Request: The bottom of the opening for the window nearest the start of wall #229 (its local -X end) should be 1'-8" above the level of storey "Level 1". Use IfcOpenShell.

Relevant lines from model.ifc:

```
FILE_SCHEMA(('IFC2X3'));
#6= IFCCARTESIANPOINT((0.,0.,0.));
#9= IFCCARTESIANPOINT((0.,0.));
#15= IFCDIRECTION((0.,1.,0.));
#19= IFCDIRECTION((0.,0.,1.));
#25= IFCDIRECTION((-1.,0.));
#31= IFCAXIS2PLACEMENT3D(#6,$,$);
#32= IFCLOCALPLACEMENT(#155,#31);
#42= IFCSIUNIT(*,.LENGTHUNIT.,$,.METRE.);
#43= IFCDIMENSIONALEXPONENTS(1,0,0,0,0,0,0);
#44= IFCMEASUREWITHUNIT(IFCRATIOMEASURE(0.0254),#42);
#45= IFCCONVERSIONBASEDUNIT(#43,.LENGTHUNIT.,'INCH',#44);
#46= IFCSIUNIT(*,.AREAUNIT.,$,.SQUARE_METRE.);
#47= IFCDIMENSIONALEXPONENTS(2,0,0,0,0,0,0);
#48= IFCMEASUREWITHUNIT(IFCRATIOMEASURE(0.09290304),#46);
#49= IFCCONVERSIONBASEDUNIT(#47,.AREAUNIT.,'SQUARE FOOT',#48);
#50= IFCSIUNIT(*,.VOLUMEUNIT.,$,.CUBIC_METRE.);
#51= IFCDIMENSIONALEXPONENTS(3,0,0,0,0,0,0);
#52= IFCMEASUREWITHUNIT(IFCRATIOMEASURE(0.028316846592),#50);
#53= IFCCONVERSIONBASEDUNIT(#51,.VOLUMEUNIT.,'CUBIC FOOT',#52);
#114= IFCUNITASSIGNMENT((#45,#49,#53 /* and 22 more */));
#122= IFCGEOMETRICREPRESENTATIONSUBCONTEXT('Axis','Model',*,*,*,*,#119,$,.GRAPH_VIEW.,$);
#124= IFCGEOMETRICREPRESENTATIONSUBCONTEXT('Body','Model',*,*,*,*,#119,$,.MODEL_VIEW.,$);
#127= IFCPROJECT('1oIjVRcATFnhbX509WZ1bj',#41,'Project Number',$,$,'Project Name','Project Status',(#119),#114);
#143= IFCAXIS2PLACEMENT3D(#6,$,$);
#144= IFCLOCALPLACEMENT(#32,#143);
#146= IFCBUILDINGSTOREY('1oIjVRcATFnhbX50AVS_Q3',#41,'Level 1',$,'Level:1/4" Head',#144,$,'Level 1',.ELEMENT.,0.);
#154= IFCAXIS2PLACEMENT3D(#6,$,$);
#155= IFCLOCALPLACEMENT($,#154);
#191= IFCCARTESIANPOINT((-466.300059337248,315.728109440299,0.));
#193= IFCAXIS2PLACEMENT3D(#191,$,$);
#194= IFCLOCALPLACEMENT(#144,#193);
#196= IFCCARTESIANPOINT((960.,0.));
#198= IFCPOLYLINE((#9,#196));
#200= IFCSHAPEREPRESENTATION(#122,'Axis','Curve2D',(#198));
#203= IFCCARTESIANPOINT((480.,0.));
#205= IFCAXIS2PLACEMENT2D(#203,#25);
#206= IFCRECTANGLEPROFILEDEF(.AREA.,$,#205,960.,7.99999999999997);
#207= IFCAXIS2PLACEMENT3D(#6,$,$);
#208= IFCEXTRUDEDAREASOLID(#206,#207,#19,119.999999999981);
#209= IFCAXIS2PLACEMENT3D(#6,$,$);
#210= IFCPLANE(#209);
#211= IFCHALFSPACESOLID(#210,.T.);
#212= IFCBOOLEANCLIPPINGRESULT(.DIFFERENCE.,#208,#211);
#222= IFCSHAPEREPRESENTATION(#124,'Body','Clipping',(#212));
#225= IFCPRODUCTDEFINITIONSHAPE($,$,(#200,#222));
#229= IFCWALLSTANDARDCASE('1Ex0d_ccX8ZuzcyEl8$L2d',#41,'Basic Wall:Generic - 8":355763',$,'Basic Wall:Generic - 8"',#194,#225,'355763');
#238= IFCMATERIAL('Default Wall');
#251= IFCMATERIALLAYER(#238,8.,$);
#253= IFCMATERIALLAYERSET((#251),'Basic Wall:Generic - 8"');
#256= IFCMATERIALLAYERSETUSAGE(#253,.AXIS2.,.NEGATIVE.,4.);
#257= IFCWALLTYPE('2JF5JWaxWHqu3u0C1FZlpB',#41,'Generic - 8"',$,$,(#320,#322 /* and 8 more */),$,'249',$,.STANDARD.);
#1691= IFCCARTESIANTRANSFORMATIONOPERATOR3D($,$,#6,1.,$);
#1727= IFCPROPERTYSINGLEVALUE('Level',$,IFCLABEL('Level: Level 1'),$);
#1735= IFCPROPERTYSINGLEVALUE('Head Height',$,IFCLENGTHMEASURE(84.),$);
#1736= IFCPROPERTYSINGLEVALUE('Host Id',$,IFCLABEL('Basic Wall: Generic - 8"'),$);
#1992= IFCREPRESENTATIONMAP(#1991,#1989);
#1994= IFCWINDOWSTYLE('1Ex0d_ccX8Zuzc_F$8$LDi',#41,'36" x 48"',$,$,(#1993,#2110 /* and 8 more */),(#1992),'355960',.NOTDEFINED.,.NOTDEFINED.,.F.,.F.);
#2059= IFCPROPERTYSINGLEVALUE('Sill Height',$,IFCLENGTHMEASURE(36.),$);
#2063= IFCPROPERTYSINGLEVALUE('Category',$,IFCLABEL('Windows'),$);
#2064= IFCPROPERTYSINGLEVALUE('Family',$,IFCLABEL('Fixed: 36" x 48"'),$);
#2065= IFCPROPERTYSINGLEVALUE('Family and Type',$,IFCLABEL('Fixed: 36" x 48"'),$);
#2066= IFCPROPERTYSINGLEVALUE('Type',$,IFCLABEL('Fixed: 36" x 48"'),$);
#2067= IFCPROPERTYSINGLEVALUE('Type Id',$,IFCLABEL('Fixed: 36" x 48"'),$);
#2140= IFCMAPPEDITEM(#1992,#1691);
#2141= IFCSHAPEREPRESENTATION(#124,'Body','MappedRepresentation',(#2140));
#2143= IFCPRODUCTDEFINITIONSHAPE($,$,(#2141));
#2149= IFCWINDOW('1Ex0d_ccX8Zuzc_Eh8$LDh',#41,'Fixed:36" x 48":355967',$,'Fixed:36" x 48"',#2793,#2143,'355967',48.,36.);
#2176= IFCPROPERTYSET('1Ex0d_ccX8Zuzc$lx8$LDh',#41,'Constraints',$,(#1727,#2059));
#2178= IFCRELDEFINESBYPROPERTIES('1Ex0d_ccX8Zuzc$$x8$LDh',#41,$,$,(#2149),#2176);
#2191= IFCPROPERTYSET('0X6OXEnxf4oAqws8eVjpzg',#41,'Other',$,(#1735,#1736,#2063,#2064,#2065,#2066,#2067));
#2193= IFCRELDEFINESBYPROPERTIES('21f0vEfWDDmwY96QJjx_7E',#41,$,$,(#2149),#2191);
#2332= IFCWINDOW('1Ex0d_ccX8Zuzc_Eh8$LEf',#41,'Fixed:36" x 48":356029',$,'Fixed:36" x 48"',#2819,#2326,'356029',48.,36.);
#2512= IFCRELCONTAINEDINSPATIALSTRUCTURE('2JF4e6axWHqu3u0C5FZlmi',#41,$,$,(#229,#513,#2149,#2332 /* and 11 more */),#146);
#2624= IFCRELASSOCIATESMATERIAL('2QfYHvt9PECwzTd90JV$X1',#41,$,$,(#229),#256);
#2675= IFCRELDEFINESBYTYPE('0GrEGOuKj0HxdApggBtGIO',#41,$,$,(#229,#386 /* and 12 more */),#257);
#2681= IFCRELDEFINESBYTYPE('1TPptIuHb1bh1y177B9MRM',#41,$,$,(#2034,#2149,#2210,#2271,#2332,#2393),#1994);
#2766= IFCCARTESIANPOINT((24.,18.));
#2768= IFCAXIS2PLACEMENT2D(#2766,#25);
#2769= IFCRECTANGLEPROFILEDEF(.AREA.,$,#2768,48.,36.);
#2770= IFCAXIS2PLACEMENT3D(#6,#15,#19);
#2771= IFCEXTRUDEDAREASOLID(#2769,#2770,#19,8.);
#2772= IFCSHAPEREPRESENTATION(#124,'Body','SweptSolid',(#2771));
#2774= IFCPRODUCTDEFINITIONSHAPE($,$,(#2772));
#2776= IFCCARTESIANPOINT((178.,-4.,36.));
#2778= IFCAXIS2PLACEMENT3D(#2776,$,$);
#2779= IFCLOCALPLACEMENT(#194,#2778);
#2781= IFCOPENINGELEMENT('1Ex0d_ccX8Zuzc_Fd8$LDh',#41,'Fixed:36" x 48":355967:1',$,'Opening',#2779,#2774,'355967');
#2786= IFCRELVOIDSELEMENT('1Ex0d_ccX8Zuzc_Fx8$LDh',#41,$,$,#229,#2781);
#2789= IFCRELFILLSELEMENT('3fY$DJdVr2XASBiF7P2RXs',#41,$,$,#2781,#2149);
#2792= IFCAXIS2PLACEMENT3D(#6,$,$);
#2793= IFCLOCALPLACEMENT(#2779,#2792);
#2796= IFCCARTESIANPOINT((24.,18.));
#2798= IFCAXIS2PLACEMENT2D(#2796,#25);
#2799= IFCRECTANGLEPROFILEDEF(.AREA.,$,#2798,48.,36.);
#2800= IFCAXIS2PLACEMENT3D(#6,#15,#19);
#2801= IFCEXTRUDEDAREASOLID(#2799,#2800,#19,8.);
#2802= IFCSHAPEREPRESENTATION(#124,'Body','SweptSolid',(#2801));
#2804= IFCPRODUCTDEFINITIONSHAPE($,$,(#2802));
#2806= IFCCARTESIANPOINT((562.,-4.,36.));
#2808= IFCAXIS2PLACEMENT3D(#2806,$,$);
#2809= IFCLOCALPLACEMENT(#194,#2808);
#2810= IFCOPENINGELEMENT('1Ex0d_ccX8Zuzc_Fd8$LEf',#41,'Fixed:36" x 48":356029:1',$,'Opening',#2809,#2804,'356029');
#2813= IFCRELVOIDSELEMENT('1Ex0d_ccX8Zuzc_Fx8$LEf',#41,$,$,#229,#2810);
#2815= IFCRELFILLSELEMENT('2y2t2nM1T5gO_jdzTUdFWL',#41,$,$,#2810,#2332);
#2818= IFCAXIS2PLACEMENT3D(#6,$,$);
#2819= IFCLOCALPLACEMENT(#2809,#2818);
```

```python
import numpy as np
import ifcopenshell
import ifcopenshell.api.geometry
import ifcopenshell.api.pset
import ifcopenshell.geom
import ifcopenshell.util.element
import ifcopenshell.util.placement
import ifcopenshell.util.shape
import ifcopenshell.util.unit

model = ifcopenshell.open("model.ifc")
unit_scale = ifcopenshell.util.unit.calculate_unit_scale(model)

window = model.by_guid("1Ex0d_ccX8Zuzc_Eh8$LDh")
opening = window.FillsVoids[0].RelatingOpeningElement
storey = ifcopenshell.util.element.get_container(window, ifc_class="IfcBuildingStorey")
level = ifcopenshell.util.placement.get_local_placement(storey.ObjectPlacement)[2, 3]

# The opening's origin need not be at the sill, so measure its lowest point.
shape = ifcopenshell.geom.create_shape(ifcopenshell.geom.settings(), opening)
bottom = ifcopenshell.util.shape.get_shape_bottom_elevation(shape, shape.geometry) / unit_scale
dz = level + 20 * 0.0254 / unit_scale - bottom

shift = np.array([0.0, 0.0, dz])
# The window is placed relative to its opening, so it follows when the opening moves.
matrix = ifcopenshell.util.placement.get_local_placement(opening.ObjectPlacement)
matrix[:3, 3] += shift
ifcopenshell.api.geometry.edit_object_placement(
    model, product=opening, matrix=matrix, is_si=False, should_transform_children=True
)

# Keep the stored heights in step.
pset = model.by_id(ifcopenshell.util.element.get_pset(window, "Constraints", should_inherit=False)["id"])
ifcopenshell.api.pset.edit_pset(model, pset=pset, properties={
    "Sill Height": model.create_entity("IfcLengthMeasure", ifcopenshell.util.element.get_pset(window, "Constraints", "Sill Height") + dz),
})
pset = model.by_id(ifcopenshell.util.element.get_pset(window, "Other", should_inherit=False)["id"])
ifcopenshell.api.pset.edit_pset(model, pset=pset, properties={
    "Head Height": model.create_entity("IfcLengthMeasure", ifcopenshell.util.element.get_pset(window, "Other", "Head Height") + dz),
})

print(f"moved by {dz * unit_scale:+.3f} m")

model.write("model_v2.ifc")
```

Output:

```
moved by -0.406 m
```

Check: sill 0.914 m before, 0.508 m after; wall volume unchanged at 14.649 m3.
